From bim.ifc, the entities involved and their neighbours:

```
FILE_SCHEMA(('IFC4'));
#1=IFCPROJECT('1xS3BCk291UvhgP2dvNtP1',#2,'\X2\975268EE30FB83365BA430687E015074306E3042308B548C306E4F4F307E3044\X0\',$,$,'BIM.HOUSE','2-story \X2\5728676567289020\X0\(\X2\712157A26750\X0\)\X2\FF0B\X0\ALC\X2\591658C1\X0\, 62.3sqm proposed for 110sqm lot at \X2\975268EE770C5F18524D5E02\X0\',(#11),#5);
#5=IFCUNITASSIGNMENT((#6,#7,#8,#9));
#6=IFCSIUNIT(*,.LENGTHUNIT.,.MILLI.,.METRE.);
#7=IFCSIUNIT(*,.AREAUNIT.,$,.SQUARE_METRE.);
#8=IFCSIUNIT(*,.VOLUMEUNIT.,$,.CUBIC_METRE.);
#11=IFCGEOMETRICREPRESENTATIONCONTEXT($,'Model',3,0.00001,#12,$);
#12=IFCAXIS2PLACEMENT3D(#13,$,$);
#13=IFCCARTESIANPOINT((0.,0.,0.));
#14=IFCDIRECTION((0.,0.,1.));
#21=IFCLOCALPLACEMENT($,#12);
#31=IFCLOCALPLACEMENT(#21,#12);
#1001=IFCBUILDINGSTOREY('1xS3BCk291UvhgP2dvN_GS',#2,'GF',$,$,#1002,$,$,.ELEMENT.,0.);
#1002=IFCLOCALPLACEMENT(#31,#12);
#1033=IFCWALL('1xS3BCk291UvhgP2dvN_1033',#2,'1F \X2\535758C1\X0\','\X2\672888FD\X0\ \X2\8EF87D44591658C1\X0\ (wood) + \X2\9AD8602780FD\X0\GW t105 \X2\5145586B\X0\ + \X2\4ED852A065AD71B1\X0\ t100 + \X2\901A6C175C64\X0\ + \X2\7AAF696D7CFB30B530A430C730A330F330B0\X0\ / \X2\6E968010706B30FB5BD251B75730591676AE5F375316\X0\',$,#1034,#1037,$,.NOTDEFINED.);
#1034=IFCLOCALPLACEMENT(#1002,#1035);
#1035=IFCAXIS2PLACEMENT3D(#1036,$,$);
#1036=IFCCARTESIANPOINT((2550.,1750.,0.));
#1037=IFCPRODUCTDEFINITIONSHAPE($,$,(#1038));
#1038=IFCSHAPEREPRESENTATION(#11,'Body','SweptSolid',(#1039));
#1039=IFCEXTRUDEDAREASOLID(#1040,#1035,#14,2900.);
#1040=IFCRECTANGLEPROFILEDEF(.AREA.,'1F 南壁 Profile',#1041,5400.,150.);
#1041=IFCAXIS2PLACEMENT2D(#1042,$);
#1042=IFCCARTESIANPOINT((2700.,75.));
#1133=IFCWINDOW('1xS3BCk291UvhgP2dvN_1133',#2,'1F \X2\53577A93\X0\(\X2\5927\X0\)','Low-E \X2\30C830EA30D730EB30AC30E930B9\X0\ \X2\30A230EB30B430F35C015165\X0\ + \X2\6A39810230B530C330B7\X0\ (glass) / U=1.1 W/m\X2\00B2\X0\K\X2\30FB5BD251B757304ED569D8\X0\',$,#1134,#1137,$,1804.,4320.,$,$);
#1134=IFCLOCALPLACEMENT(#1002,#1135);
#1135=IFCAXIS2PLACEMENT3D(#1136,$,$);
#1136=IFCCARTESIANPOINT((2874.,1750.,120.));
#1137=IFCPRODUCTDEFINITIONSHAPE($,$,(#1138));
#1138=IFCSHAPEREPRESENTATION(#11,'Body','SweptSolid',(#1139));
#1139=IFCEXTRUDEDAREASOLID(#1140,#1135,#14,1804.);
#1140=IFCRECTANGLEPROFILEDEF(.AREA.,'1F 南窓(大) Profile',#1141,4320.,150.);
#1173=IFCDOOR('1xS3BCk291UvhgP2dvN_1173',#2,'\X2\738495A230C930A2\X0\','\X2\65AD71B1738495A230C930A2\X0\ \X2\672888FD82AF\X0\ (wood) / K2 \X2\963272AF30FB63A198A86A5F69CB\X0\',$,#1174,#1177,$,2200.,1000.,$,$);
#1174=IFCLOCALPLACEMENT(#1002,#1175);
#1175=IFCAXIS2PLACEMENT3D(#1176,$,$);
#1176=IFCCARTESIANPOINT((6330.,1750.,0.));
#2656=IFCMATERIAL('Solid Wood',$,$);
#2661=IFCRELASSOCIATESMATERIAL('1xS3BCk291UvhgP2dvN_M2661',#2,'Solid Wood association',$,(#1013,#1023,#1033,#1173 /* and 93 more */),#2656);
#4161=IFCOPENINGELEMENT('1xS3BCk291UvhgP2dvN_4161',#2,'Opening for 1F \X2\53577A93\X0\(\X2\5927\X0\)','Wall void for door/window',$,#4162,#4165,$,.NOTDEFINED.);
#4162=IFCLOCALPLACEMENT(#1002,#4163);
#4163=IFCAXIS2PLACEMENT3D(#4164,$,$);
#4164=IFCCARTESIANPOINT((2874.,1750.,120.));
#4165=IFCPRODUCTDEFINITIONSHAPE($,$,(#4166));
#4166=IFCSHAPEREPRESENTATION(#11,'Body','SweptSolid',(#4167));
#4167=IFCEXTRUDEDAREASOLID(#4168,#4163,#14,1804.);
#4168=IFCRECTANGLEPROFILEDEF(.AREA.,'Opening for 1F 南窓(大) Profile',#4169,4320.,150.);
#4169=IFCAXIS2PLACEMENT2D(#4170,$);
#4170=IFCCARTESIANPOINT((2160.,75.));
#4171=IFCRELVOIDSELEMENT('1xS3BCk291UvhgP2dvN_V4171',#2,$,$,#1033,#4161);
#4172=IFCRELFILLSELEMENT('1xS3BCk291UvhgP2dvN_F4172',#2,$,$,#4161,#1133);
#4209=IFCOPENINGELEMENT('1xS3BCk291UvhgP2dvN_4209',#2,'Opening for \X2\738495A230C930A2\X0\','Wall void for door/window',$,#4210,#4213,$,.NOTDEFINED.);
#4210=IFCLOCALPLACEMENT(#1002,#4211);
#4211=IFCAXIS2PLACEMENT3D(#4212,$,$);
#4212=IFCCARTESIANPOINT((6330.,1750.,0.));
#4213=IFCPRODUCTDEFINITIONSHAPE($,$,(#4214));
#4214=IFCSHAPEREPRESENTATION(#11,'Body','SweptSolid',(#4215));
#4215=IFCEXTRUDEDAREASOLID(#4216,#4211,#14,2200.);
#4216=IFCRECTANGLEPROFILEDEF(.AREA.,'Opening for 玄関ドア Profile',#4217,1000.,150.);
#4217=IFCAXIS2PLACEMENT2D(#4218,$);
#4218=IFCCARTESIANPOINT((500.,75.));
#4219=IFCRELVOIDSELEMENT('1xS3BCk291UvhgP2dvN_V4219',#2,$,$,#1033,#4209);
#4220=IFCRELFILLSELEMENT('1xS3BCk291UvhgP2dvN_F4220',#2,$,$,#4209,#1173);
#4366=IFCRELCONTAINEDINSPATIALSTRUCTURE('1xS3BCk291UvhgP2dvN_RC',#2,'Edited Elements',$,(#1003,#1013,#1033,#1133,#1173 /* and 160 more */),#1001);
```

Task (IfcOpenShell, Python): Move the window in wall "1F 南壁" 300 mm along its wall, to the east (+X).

```python
import ifcopenshell
import ifcopenshell.api.geometry
import ifcopenshell.util.placement
import ifcopenshell.util.unit

model = ifcopenshell.open("bim.ifc")
unit_scale = ifcopenshell.util.unit.calculate_unit_scale(model)

window = model.by_id(1133)
opening = window.FillsVoids[0].RelatingOpeningElement
wall = opening.VoidsElements[0].RelatingBuildingElement

wall_matrix = ifcopenshell.util.placement.get_local_placement(wall.ObjectPlacement)
shift = wall_matrix[:3, 0] * 0.3 / unit_scale
before = ifcopenshell.util.placement.get_local_placement(window.ObjectPlacement)[:3, 3].copy()

# The window is not placed relative to its opening, so move both.
for product in (opening, window):
    matrix = ifcopenshell.util.placement.get_local_placement(product.ObjectPlacement)
    matrix[:3, 3] += shift
    ifcopenshell.api.geometry.edit_object_placement(model, product=product, matrix=matrix, is_si=False)

after = ifcopenshell.util.placement.get_local_placement(window.ObjectPlacement)[:3, 3]
print("window moved by", (after - before).round(3) + 0.0)

model.write("bim_v2.ifc")
```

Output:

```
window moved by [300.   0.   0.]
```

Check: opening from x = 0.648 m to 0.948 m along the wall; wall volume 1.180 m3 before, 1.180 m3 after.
